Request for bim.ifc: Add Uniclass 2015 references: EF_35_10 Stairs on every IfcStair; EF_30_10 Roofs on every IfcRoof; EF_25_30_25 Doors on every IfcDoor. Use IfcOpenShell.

First a look at what the model holds.

```python
import ifcopenshell

model = ifcopenshell.open("bim.ifc")
print(model.schema)
print("classifications:", [c.Name for c in model.by_type("IfcClassification")])
for ifc_class in ("IfcDoor", "IfcRoof", "IfcStair", "IfcWall", "IfcWindow"):
    print(ifc_class, len(model.by_type(ifc_class)))
```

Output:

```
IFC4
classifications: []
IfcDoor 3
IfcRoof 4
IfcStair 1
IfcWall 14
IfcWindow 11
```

```python
import ifcopenshell
import ifcopenshell.api.classification

model = ifcopenshell.open("bim.ifc")

system = ifcopenshell.api.classification.add_classification(model, classification="Uniclass 2015")

codes = {
    "IfcStair": ("EF_35_10", "Stairs"),
    "IfcRoof": ("EF_30_10", "Roofs"),
    "IfcDoor": ("EF_25_30_25", "Doors"),
}
for ifc_class, (code, name) in codes.items():
    products = model.by_type(ifc_class)
    ifcopenshell.api.classification.add_reference(
        model, products=products, classification=system, identification=code, name=name
    )
    print(code, len(products))

model.write("bim_updated.ifc")
```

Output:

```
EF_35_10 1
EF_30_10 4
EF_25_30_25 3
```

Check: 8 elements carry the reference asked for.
